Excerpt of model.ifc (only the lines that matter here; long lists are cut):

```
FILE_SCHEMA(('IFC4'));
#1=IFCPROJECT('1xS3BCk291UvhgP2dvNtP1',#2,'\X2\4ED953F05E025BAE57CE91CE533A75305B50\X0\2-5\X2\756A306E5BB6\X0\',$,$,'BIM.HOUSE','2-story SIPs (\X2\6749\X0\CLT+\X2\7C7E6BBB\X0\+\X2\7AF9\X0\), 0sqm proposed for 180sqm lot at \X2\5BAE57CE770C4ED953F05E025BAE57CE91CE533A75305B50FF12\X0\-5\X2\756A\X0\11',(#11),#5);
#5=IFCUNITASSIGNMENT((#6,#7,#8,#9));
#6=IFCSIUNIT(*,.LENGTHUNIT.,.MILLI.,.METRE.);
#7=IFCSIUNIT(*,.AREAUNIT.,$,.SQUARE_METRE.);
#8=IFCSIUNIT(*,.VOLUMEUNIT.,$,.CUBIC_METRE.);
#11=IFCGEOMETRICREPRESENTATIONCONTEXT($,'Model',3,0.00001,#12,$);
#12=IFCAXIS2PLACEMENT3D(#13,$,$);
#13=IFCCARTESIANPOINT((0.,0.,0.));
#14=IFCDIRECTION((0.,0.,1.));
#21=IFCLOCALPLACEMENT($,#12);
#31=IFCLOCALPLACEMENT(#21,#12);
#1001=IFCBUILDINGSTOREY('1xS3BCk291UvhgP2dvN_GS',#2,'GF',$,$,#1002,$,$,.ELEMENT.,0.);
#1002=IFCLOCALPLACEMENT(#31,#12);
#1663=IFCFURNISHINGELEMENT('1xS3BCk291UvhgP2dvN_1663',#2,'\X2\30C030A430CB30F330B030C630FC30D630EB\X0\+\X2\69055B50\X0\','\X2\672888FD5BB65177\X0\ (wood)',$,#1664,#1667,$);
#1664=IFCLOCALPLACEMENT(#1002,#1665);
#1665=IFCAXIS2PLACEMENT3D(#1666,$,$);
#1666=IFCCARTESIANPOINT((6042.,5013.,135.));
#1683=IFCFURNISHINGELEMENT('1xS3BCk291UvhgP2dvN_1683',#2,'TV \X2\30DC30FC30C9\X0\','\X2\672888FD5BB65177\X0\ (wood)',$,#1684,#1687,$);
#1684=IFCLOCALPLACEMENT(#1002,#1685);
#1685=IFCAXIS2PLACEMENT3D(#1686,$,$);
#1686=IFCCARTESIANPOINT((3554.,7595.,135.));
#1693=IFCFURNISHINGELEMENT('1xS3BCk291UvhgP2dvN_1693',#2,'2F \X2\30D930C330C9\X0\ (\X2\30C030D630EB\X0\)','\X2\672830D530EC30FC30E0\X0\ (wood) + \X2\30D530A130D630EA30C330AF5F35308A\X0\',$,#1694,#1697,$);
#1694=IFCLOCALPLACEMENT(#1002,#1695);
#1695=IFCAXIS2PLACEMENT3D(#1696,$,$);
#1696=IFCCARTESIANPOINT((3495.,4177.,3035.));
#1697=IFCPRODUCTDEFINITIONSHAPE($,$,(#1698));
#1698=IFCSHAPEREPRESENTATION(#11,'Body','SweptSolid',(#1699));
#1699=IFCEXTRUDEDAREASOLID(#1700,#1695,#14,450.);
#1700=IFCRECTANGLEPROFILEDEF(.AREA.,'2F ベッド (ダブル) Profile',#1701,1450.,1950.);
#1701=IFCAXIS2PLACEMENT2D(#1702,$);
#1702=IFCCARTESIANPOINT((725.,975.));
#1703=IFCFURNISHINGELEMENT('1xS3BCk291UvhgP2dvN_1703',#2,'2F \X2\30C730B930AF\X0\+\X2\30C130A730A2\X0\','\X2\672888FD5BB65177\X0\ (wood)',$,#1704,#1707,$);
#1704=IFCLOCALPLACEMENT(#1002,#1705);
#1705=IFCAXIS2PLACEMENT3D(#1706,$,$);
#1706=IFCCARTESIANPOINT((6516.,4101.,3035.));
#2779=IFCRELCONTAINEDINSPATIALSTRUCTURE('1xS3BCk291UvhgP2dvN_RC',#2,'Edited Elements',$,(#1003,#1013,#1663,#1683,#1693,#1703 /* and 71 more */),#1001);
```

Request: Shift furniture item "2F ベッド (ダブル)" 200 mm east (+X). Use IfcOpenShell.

```python
import ifcopenshell
import ifcopenshell.api.geometry
import ifcopenshell.util.placement

model = ifcopenshell.open("model.ifc")

item = model.by_id(1693)
matrix = ifcopenshell.util.placement.get_local_placement(item.ObjectPlacement)
matrix[0, 3] += 200.0
ifcopenshell.api.geometry.edit_object_placement(model, product=item, matrix=matrix, is_si=False)

print(ifcopenshell.util.placement.get_local_placement(item.ObjectPlacement).round(3) + 0.0)

model.write("model_edited.ifc")
```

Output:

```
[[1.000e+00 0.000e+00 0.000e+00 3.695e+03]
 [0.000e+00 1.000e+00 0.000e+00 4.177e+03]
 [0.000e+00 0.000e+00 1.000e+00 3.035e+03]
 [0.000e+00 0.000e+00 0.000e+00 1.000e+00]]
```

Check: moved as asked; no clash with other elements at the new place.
